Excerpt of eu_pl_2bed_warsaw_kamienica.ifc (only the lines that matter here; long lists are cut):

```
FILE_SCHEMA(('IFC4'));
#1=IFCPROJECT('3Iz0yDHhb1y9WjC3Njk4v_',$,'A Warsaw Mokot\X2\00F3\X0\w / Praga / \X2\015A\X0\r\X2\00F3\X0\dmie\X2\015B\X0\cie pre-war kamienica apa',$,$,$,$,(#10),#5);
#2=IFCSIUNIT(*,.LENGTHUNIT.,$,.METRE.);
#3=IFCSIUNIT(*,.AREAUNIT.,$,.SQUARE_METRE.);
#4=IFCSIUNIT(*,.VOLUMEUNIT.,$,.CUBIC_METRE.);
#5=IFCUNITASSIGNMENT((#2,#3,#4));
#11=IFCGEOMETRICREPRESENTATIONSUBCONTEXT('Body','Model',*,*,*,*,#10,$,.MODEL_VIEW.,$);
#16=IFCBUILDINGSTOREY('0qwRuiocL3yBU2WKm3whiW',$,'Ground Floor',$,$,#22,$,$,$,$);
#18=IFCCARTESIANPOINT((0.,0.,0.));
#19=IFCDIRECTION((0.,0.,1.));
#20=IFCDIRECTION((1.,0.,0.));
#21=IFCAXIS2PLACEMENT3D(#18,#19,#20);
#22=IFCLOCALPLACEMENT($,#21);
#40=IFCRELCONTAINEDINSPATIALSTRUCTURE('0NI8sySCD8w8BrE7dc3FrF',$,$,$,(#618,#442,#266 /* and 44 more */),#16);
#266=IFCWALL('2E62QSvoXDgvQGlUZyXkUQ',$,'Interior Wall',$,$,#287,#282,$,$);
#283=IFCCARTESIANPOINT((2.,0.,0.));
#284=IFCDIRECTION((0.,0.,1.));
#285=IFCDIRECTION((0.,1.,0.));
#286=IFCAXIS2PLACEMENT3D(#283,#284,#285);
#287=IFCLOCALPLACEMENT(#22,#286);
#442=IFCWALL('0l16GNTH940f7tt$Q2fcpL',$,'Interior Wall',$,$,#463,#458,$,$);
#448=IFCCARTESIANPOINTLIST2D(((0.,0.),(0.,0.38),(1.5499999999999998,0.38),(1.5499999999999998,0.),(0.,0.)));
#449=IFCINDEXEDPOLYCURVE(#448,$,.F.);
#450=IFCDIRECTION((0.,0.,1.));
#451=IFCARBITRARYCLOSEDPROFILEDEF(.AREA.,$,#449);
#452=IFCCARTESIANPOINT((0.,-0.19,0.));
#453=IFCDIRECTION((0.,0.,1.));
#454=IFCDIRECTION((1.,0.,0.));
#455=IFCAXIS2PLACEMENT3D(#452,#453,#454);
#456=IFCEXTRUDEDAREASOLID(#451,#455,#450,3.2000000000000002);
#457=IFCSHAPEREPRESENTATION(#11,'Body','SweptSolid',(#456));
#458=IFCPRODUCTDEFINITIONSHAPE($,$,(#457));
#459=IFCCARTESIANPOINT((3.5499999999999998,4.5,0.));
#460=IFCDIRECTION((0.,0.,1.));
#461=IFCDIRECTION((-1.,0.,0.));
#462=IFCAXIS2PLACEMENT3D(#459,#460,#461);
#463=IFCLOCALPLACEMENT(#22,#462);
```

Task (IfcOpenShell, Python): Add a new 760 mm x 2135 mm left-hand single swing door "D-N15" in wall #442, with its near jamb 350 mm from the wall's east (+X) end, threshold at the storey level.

```python
import numpy as np
import ifcopenshell
import ifcopenshell.api.feature
import ifcopenshell.api.geometry
import ifcopenshell.api.root
import ifcopenshell.api.spatial
import ifcopenshell.geom
import ifcopenshell.util.element
import ifcopenshell.util.placement
import ifcopenshell.util.representation
import ifcopenshell.util.shape
import ifcopenshell.util.unit

model = ifcopenshell.open("eu_pl_2bed_warsaw_kamienica.ifc")
unit_scale = ifcopenshell.util.unit.calculate_unit_scale(model)
settings = ifcopenshell.geom.settings()


def volume(element):
    """Net volume in cubic metres, openings subtracted."""
    shape = ifcopenshell.geom.create_shape(settings, element)
    return ifcopenshell.util.shape.get_volume(shape.geometry)


wall = model.by_guid("0l16GNTH940f7tt$Q2fcpL")
storey = ifcopenshell.util.element.get_container(wall, ifc_class="IfcBuildingStorey")
context = ifcopenshell.util.representation.get_context(model, "Model", "Body", "MODEL_VIEW")
before = volume(wall)

width, height, from_end, sill = 0.76, 2.135, 0.35, 0.0  # metres

# The wall runs along its own X axis, and the end named is its -X end.
wall_shape = ifcopenshell.geom.create_shape(settings, wall)
x, y, z = ifcopenshell.util.shape.get_vertices(wall_shape.geometry).T
start = x.min() + from_end
face, thickness = float(y.min()), float(y.max() - y.min())
wall_matrix = ifcopenshell.util.placement.get_local_placement(wall.ObjectPlacement)
level = ifcopenshell.util.placement.get_local_placement(storey.ObjectPlacement)[2, 3]


def in_wall(x, y):
    """Placement at x, y metres in the wall's axes, at sill height."""
    matrix = wall_matrix.copy()
    matrix[:, 3] = wall_matrix @ np.array([x / unit_scale, y / unit_scale, 0.0, 1.0])
    matrix[2, 3] = level + sill / unit_scale
    return matrix


# Opening: a box that overshoots both wall faces by 50 mm.
opening = ifcopenshell.api.root.create_entity(model, ifc_class="IfcOpeningElement", predefined_type="OPENING")
box = ifcopenshell.api.geometry.add_wall_representation(
    model, context=context, length=width, height=height, thickness=thickness + 0.1
)
ifcopenshell.api.geometry.assign_representation(model, product=opening, representation=box)
ifcopenshell.api.geometry.edit_object_placement(model, product=opening, matrix=in_wall(start, face - 0.05), is_si=False)
ifcopenshell.api.feature.add_feature(model, feature=opening, element=wall)

door = ifcopenshell.api.root.create_entity(model, ifc_class="IfcDoor", name="D-N15", predefined_type="DOOR")
door.OverallWidth, door.OverallHeight = width / unit_scale, height / unit_scale
door.OperationType = "SINGLE_SWING_LEFT"
body = ifcopenshell.api.geometry.add_door_representation(
    model,
    context=context,
    overall_width=door.OverallWidth,
    overall_height=door.OverallHeight,
    operation_type="SINGLE_SWING_LEFT",
    lining_properties={"LiningDepth": thickness / unit_scale, "ThresholdDepth": thickness / unit_scale},
)
ifcopenshell.api.geometry.assign_representation(model, product=door, representation=body)
ifcopenshell.api.spatial.assign_container(model, products=[door], relating_structure=storey)
ifcopenshell.api.feature.add_filling(model, opening=opening, element=door)

# The lining spans the wall, so the door starts at the wall face.
ifcopenshell.api.geometry.edit_object_placement(model, product=door, matrix=in_wall(start, face), is_si=False)

after = volume(wall)

print(f"wall volume {before:.3f} -> {after:.3f} m3")

model.write("eu_pl_2bed_warsaw_kamienica_updated.ifc")
```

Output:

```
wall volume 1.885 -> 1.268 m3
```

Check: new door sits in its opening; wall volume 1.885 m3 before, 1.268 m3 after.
